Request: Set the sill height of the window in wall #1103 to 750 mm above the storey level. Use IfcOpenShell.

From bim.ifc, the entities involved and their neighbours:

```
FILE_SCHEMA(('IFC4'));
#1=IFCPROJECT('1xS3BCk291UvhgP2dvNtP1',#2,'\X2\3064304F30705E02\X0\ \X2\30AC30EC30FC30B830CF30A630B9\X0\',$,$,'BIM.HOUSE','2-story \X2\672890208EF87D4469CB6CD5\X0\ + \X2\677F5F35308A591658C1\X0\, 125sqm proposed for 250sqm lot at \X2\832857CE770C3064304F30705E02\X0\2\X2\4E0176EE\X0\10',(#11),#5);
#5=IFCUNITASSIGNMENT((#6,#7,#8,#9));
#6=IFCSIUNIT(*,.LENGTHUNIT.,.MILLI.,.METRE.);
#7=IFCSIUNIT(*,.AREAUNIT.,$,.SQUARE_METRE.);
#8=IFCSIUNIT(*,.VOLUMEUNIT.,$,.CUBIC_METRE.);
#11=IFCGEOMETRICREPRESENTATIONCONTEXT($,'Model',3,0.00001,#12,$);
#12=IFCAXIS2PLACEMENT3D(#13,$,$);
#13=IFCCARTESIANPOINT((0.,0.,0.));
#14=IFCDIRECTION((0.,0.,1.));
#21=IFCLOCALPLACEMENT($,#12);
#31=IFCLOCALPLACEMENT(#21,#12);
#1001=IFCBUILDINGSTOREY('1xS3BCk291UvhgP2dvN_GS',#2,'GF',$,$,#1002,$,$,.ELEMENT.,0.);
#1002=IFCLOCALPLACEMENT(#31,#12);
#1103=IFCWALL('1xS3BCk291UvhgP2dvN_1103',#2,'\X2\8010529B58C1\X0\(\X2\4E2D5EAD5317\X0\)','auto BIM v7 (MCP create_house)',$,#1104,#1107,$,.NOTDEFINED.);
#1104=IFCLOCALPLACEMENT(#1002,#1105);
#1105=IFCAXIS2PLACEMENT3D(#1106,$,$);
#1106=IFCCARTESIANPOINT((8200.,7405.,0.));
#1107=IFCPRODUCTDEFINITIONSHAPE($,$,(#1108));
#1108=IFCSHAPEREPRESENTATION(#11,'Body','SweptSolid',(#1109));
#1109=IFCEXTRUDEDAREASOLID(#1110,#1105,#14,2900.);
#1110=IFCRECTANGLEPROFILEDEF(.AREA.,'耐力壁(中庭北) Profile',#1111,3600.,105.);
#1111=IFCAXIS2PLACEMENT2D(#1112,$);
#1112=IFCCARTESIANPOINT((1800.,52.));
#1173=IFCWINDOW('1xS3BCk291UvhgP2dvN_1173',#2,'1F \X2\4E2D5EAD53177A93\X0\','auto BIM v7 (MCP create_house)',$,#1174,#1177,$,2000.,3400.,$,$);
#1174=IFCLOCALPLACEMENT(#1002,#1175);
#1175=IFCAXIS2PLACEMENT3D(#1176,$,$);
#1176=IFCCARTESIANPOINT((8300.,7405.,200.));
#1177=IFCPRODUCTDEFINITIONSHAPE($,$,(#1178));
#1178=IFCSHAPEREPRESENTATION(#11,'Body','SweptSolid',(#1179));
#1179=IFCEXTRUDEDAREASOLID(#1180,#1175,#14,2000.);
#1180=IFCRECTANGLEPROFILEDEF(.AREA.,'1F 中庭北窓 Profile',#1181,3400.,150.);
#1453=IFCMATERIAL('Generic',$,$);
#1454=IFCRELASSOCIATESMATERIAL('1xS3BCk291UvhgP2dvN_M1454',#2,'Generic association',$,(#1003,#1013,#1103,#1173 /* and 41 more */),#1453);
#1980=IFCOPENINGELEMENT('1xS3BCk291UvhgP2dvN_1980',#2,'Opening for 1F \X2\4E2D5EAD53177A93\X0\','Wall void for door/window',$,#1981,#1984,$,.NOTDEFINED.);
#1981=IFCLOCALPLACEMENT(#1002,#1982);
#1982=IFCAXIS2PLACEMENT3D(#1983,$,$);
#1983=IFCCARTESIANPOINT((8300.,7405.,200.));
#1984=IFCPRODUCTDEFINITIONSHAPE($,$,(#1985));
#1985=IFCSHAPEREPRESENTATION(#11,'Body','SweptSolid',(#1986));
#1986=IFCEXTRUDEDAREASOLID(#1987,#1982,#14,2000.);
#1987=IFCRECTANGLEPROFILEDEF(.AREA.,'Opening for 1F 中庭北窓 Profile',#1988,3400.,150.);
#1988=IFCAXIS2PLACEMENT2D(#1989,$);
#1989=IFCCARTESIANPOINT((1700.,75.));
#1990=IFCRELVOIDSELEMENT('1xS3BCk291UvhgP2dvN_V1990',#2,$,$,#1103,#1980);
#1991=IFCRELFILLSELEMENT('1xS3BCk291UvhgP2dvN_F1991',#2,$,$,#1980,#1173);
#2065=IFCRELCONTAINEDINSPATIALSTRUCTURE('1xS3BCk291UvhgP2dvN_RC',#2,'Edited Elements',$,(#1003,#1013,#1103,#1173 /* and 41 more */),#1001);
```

```python
import numpy as np
import ifcopenshell
import ifcopenshell.api.geometry
import ifcopenshell.geom
import ifcopenshell.util.element
import ifcopenshell.util.placement
import ifcopenshell.util.shape
import ifcopenshell.util.unit

model = ifcopenshell.open("bim.ifc")
unit_scale = ifcopenshell.util.unit.calculate_unit_scale(model)

window = model.by_guid("1xS3BCk291UvhgP2dvN_1173")
opening = window.FillsVoids[0].RelatingOpeningElement
storey = ifcopenshell.util.element.get_container(window, ifc_class="IfcBuildingStorey")
level = ifcopenshell.util.placement.get_local_placement(storey.ObjectPlacement)[2, 3]

# The opening's origin need not be at the sill, so measure its lowest point.
shape = ifcopenshell.geom.create_shape(ifcopenshell.geom.settings(), opening)
bottom = ifcopenshell.util.shape.get_shape_bottom_elevation(shape, shape.geometry) / unit_scale
dz = level + 0.75 / unit_scale - bottom

shift = np.array([0.0, 0.0, dz])
# The window is not placed relative to its opening, so move both.
for product in (opening, window):
    matrix = ifcopenshell.util.placement.get_local_placement(product.ObjectPlacement)
    matrix[:3, 3] += shift
    ifcopenshell.api.geometry.edit_object_placement(model, product=product, matrix=matrix, is_si=False)

print(f"moved by {dz * unit_scale:+.3f} m")

model.write("bim_rev.ifc")
```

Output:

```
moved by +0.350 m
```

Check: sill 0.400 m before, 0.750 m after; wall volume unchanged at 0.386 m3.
